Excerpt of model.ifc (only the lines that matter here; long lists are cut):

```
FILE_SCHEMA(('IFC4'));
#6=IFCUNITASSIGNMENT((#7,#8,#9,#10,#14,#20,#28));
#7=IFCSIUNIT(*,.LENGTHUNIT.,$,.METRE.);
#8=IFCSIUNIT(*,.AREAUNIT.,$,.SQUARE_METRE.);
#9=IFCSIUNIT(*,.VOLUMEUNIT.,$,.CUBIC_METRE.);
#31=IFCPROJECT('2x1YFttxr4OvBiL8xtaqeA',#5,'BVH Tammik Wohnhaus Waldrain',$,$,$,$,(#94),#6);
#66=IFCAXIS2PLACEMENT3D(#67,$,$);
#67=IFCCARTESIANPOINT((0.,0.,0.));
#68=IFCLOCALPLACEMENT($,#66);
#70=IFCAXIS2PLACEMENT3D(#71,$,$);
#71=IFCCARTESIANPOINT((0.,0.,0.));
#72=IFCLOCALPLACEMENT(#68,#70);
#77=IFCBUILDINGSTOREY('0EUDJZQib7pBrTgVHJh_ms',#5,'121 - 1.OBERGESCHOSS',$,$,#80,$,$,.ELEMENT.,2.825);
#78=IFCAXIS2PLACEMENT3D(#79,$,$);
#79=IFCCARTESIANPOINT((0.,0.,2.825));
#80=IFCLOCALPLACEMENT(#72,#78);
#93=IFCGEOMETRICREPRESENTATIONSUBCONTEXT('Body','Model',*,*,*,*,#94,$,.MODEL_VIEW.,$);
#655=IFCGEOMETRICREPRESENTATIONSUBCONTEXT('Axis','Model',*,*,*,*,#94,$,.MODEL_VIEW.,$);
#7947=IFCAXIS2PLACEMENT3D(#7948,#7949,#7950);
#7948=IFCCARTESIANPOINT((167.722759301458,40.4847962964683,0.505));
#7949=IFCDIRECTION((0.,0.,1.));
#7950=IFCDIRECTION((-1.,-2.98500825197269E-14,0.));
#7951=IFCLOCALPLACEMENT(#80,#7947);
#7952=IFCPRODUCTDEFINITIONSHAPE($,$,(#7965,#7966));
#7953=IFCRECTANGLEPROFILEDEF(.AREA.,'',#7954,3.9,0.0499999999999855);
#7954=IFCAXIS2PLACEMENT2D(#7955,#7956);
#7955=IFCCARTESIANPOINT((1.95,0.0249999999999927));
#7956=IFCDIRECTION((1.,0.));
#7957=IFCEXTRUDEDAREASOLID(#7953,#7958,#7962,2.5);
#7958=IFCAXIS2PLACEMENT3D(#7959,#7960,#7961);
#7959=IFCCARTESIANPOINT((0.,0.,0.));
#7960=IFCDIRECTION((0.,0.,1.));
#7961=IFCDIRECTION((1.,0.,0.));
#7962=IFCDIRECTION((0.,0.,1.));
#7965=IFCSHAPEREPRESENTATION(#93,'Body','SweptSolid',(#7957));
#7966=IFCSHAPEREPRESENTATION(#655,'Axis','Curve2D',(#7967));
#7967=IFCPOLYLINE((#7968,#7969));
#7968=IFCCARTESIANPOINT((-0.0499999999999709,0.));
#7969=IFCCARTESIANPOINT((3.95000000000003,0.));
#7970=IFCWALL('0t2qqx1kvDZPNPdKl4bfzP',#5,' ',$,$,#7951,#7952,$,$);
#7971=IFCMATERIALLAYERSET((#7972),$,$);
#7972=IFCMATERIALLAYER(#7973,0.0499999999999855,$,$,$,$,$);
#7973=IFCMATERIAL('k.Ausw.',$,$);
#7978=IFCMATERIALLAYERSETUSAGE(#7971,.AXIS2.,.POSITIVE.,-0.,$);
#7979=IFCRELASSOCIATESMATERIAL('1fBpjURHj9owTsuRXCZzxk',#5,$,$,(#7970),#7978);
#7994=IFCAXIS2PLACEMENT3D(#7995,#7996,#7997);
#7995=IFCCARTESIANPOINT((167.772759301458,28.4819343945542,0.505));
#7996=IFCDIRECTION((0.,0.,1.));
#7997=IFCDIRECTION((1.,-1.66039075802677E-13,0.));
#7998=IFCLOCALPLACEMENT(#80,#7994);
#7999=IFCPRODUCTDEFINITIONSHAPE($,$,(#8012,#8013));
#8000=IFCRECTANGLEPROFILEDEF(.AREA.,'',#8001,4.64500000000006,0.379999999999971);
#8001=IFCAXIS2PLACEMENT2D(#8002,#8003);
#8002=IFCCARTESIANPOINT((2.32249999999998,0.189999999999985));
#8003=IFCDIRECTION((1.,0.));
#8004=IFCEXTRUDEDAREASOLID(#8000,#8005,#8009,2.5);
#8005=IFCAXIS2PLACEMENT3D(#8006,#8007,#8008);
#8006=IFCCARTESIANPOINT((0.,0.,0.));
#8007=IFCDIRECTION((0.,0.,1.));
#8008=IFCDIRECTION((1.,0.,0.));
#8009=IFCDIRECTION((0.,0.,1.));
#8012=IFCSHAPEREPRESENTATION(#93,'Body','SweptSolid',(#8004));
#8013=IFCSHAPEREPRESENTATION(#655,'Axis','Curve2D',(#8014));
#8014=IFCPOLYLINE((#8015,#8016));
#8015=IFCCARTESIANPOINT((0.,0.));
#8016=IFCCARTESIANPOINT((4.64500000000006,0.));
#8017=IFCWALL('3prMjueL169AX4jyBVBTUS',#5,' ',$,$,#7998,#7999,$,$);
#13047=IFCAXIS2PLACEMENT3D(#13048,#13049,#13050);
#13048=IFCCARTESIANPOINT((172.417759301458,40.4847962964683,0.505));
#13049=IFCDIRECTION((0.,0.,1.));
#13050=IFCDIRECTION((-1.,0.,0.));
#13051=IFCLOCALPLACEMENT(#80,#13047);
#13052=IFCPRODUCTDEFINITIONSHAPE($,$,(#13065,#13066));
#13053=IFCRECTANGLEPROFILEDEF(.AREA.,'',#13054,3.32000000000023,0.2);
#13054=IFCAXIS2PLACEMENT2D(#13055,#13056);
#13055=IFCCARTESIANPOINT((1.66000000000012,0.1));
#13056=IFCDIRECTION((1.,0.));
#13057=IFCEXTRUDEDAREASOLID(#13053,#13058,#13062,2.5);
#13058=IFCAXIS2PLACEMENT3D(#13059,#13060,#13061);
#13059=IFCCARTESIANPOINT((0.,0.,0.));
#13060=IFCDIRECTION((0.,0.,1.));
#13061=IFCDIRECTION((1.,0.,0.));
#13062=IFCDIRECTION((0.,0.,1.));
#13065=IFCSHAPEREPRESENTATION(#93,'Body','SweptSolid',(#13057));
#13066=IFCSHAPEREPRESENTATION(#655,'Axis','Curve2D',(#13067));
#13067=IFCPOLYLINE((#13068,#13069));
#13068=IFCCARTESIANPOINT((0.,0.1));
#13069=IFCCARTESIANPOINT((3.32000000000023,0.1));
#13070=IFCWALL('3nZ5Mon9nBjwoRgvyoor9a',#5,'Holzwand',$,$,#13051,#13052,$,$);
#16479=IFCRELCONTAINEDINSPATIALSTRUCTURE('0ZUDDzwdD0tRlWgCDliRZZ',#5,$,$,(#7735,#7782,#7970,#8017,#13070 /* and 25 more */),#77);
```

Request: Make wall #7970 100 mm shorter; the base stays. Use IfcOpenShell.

```python
import ifcopenshell
import ifcopenshell.geom
import ifcopenshell.util.representation
import ifcopenshell.util.shape

model = ifcopenshell.open("model.ifc")
settings = ifcopenshell.geom.settings()


def volume(element):
    """Net volume in cubic metres, openings subtracted."""
    shape = ifcopenshell.geom.create_shape(settings, element)
    return ifcopenshell.util.shape.get_volume(shape.geometry)


wall = model.by_guid("0t2qqx1kvDZPNPdKl4bfzP")
before = volume(wall)

body = ifcopenshell.util.representation.get_representation(wall, "Model", "Body")
solid = body.Items[0]
old_height = solid.Depth
solid.Depth -= 0.1
after = volume(wall)

print(f"height {old_height:g} -> {solid.Depth:g}, volume {before:.3f} -> {after:.3f} m3")

model.write("model-out.ifc")
```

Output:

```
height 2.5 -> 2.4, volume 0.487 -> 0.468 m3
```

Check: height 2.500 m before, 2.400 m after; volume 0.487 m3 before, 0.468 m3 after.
